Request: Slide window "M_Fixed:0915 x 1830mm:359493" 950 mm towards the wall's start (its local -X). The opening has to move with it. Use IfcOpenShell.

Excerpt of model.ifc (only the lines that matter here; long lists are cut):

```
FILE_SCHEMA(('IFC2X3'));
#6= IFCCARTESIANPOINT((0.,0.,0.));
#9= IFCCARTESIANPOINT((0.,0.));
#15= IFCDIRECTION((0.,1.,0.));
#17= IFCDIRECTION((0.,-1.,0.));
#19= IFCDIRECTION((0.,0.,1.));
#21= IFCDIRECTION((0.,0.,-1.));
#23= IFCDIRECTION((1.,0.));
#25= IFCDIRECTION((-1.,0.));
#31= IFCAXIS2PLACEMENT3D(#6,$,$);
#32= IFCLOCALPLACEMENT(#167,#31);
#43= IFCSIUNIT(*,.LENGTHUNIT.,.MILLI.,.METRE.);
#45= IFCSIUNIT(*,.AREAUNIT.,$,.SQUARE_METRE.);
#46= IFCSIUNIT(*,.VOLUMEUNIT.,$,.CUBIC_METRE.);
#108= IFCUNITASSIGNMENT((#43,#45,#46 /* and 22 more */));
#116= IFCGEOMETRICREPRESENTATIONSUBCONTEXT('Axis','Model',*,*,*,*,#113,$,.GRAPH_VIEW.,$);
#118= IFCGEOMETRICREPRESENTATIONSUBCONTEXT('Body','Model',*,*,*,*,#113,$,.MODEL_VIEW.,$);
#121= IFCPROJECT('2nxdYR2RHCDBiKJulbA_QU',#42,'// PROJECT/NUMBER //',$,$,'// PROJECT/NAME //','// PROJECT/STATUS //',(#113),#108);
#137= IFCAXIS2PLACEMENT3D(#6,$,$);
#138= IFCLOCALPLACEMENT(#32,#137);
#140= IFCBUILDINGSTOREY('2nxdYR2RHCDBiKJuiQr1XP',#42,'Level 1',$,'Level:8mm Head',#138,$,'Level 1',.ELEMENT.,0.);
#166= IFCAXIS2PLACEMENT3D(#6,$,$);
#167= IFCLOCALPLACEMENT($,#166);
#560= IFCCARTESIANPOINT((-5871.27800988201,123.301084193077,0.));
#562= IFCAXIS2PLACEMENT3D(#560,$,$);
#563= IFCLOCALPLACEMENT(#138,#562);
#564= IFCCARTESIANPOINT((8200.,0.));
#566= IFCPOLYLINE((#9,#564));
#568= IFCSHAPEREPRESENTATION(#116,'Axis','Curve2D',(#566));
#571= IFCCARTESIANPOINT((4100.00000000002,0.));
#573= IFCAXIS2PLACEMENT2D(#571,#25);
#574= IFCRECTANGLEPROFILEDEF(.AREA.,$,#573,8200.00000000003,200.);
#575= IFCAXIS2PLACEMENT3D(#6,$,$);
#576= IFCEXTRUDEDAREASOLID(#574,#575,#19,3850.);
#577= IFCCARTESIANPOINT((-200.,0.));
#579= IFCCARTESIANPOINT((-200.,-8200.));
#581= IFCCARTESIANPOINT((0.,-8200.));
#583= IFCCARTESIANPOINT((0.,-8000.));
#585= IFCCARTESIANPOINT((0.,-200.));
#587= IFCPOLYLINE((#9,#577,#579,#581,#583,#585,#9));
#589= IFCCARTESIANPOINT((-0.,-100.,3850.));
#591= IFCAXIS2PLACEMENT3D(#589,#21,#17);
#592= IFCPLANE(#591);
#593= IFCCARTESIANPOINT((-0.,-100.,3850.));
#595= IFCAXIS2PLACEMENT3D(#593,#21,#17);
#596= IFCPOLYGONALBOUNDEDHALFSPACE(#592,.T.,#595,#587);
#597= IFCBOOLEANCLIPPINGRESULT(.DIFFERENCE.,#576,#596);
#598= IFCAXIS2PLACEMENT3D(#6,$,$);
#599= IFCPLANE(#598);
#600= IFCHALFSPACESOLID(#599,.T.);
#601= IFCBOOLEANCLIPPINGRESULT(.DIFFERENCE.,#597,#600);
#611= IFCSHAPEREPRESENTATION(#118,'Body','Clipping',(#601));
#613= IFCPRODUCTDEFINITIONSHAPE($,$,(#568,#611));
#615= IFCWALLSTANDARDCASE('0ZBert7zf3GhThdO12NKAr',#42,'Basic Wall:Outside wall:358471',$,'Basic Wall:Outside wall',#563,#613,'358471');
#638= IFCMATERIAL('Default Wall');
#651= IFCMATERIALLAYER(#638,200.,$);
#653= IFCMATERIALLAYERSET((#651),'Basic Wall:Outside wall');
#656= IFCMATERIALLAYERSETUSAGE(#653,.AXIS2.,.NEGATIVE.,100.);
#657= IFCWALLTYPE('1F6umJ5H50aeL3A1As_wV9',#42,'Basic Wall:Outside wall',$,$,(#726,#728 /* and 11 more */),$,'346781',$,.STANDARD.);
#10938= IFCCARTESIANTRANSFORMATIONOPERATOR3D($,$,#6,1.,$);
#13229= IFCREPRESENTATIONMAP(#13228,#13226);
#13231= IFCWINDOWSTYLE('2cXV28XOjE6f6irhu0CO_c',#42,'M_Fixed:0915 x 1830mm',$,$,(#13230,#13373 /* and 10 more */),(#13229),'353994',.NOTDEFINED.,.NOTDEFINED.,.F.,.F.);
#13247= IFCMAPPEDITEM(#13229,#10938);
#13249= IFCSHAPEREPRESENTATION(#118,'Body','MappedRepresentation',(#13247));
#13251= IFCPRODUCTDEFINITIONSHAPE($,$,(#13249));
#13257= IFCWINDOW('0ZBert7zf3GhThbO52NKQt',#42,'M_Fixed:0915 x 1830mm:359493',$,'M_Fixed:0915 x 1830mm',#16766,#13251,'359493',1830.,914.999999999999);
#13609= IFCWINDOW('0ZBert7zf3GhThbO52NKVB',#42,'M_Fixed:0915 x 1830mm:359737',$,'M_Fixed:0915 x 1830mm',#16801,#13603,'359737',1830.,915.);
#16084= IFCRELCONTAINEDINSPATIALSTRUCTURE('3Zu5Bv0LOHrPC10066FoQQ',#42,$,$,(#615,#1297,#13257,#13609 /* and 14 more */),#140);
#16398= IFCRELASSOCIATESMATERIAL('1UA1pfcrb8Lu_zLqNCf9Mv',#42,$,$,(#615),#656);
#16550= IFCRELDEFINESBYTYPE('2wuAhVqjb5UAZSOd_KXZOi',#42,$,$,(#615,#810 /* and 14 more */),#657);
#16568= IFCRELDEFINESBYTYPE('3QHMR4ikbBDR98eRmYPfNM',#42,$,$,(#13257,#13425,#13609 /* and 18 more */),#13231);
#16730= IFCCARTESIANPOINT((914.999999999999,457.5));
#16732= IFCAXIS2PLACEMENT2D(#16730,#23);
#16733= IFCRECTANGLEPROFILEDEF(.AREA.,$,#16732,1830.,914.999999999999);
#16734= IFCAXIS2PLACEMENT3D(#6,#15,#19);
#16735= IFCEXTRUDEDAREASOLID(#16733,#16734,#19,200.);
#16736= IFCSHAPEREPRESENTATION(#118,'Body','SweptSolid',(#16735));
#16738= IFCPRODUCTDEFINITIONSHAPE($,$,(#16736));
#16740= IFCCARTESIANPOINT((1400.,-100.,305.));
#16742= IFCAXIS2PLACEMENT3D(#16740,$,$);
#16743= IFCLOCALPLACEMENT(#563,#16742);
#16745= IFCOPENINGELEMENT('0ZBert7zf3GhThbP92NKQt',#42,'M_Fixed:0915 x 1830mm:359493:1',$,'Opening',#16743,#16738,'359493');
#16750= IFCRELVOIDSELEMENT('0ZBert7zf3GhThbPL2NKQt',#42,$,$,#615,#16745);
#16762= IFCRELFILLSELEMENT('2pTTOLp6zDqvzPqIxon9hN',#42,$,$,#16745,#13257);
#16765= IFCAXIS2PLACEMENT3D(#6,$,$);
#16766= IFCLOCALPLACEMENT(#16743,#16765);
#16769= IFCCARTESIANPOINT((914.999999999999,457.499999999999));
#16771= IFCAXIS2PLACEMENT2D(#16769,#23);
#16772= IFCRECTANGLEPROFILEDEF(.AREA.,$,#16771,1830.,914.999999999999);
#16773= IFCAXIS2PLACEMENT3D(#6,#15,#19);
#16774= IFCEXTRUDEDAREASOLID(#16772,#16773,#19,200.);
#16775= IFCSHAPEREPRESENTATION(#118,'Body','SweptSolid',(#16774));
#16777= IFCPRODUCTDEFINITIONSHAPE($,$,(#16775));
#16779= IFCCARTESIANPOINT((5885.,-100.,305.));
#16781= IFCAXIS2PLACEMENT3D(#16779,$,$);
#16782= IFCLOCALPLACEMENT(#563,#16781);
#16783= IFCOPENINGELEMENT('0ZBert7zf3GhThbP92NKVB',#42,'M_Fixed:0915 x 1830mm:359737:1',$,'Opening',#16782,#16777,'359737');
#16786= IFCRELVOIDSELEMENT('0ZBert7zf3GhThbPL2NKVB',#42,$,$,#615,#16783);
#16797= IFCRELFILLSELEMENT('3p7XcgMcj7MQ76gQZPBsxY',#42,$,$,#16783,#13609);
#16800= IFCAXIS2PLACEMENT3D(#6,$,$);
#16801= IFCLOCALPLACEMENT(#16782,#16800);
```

```python
import ifcopenshell
import ifcopenshell.api.geometry
import ifcopenshell.util.placement

model = ifcopenshell.open("model.ifc")

window = model.by_id(13257)
opening = window.FillsVoids[0].RelatingOpeningElement
wall = opening.VoidsElements[0].RelatingBuildingElement

wall_matrix = ifcopenshell.util.placement.get_local_placement(wall.ObjectPlacement)
shift = wall_matrix[:3, 0] * -950.0
before = ifcopenshell.util.placement.get_local_placement(window.ObjectPlacement)[:3, 3].copy()

# The window is placed relative to its opening, so it follows when the opening moves.
matrix = ifcopenshell.util.placement.get_local_placement(opening.ObjectPlacement)
matrix[:3, 3] += shift
ifcopenshell.api.geometry.edit_object_placement(
    model, product=opening, matrix=matrix, is_si=False, should_transform_children=True
)

after = ifcopenshell.util.placement.get_local_placement(window.ObjectPlacement)[:3, 3]
print("window moved by", (after - before).round(3) + 0.0)

model.write("model_edited.ifc")
```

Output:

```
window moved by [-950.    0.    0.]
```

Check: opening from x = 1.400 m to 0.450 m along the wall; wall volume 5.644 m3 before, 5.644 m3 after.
